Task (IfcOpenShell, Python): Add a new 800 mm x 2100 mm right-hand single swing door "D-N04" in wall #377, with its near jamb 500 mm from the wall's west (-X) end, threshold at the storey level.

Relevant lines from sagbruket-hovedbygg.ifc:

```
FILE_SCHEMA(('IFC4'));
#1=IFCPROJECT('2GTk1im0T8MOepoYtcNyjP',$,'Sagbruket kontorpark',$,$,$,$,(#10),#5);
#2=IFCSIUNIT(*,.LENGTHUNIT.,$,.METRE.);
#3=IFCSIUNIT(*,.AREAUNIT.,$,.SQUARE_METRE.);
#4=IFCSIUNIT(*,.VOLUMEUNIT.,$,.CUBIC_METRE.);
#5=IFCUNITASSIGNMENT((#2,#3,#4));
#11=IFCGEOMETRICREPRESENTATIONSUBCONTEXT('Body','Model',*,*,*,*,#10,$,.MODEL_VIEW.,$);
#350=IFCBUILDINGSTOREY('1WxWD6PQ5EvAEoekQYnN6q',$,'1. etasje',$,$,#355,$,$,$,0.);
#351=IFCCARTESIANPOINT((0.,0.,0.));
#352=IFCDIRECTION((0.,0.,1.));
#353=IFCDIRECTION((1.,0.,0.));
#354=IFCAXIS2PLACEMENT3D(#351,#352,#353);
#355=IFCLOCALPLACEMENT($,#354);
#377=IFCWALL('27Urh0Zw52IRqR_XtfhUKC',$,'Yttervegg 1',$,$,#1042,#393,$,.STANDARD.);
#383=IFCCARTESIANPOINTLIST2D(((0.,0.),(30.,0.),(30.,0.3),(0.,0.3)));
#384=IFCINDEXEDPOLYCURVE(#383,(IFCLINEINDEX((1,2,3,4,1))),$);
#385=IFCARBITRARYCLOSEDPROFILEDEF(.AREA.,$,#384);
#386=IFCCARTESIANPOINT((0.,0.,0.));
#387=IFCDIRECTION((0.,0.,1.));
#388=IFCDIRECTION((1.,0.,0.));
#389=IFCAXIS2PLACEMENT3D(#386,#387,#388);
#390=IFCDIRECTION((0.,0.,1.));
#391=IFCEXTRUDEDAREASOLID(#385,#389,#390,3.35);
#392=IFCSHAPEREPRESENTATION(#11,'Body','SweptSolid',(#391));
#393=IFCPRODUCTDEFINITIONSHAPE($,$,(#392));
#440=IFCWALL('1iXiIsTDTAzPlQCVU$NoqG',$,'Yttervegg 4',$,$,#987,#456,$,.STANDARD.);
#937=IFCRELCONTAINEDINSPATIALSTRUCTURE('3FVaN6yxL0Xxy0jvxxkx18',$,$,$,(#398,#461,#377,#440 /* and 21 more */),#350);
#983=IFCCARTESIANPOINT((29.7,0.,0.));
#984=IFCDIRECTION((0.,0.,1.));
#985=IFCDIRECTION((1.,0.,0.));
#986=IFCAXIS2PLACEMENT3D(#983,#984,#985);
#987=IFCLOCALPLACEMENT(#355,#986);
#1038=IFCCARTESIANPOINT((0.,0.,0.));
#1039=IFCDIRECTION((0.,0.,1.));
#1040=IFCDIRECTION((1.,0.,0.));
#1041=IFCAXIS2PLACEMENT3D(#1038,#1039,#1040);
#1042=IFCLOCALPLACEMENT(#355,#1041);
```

```python
import numpy as np
import ifcopenshell
import ifcopenshell.api.feature
import ifcopenshell.api.geometry
import ifcopenshell.api.root
import ifcopenshell.api.spatial
import ifcopenshell.geom
import ifcopenshell.util.element
import ifcopenshell.util.placement
import ifcopenshell.util.representation
import ifcopenshell.util.shape
import ifcopenshell.util.unit

model = ifcopenshell.open("sagbruket-hovedbygg.ifc")
unit_scale = ifcopenshell.util.unit.calculate_unit_scale(model)
settings = ifcopenshell.geom.settings()


def volume(element):
    """Net volume in cubic metres, openings subtracted."""
    shape = ifcopenshell.geom.create_shape(settings, element)
    return ifcopenshell.util.shape.get_volume(shape.geometry)


wall = model.by_guid("27Urh0Zw52IRqR_XtfhUKC")
storey = ifcopenshell.util.element.get_container(wall, ifc_class="IfcBuildingStorey")
context = ifcopenshell.util.representation.get_context(model, "Model", "Body", "MODEL_VIEW")
before = volume(wall)

width, height, from_end, sill = 0.8, 2.1, 0.5, 0.0  # metres

# The wall runs along its own X axis, and the end named is its -X end.
wall_shape = ifcopenshell.geom.create_shape(settings, wall)
x, y, z = ifcopenshell.util.shape.get_vertices(wall_shape.geometry).T
start = x.min() + from_end
face, thickness = float(y.min()), float(y.max() - y.min())
wall_matrix = ifcopenshell.util.placement.get_local_placement(wall.ObjectPlacement)
level = ifcopenshell.util.placement.get_local_placement(storey.ObjectPlacement)[2, 3]


def in_wall(x, y):
    """Placement at x, y metres in the wall's axes, at sill height."""
    matrix = wall_matrix.copy()
    matrix[:, 3] = wall_matrix @ np.array([x / unit_scale, y / unit_scale, 0.0, 1.0])
    matrix[2, 3] = level + sill / unit_scale
    return matrix


# Opening: a box that overshoots both wall faces by 50 mm.
opening = ifcopenshell.api.root.create_entity(model, ifc_class="IfcOpeningElement", predefined_type="OPENING")
box = ifcopenshell.api.geometry.add_wall_representation(
    model, context=context, length=width, height=height, thickness=thickness + 0.1
)
ifcopenshell.api.geometry.assign_representation(model, product=opening, representation=box)
ifcopenshell.api.geometry.edit_object_placement(model, product=opening, matrix=in_wall(start, face - 0.05), is_si=False)
ifcopenshell.api.feature.add_feature(model, feature=opening, element=wall)

door = ifcopenshell.api.root.create_entity(model, ifc_class="IfcDoor", name="D-N04", predefined_type="DOOR")
door.OverallWidth, door.OverallHeight = width / unit_scale, height / unit_scale
door.OperationType = "SINGLE_SWING_RIGHT"
body = ifcopenshell.api.geometry.add_door_representation(
    model,
    context=context,
    overall_width=door.OverallWidth,
    overall_height=door.OverallHeight,
    operation_type="SINGLE_SWING_RIGHT",
    lining_properties={"LiningDepth": thickness / unit_scale, "ThresholdDepth": thickness / unit_scale},
)
ifcopenshell.api.geometry.assign_representation(model, product=door, representation=body)
ifcopenshell.api.spatial.assign_container(model, products=[door], relating_structure=storey)
ifcopenshell.api.feature.add_filling(model, opening=opening, element=door)

# The lining spans the wall, so the door starts at the wall face.
ifcopenshell.api.geometry.edit_object_placement(model, product=door, matrix=in_wall(start, face), is_si=False)

after = volume(wall)

print(f"wall volume {before:.3f} -> {after:.3f} m3")

model.write("sagbruket-hovedbygg_rev.ifc")
```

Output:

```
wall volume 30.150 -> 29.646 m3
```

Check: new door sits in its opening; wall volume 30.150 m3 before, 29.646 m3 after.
